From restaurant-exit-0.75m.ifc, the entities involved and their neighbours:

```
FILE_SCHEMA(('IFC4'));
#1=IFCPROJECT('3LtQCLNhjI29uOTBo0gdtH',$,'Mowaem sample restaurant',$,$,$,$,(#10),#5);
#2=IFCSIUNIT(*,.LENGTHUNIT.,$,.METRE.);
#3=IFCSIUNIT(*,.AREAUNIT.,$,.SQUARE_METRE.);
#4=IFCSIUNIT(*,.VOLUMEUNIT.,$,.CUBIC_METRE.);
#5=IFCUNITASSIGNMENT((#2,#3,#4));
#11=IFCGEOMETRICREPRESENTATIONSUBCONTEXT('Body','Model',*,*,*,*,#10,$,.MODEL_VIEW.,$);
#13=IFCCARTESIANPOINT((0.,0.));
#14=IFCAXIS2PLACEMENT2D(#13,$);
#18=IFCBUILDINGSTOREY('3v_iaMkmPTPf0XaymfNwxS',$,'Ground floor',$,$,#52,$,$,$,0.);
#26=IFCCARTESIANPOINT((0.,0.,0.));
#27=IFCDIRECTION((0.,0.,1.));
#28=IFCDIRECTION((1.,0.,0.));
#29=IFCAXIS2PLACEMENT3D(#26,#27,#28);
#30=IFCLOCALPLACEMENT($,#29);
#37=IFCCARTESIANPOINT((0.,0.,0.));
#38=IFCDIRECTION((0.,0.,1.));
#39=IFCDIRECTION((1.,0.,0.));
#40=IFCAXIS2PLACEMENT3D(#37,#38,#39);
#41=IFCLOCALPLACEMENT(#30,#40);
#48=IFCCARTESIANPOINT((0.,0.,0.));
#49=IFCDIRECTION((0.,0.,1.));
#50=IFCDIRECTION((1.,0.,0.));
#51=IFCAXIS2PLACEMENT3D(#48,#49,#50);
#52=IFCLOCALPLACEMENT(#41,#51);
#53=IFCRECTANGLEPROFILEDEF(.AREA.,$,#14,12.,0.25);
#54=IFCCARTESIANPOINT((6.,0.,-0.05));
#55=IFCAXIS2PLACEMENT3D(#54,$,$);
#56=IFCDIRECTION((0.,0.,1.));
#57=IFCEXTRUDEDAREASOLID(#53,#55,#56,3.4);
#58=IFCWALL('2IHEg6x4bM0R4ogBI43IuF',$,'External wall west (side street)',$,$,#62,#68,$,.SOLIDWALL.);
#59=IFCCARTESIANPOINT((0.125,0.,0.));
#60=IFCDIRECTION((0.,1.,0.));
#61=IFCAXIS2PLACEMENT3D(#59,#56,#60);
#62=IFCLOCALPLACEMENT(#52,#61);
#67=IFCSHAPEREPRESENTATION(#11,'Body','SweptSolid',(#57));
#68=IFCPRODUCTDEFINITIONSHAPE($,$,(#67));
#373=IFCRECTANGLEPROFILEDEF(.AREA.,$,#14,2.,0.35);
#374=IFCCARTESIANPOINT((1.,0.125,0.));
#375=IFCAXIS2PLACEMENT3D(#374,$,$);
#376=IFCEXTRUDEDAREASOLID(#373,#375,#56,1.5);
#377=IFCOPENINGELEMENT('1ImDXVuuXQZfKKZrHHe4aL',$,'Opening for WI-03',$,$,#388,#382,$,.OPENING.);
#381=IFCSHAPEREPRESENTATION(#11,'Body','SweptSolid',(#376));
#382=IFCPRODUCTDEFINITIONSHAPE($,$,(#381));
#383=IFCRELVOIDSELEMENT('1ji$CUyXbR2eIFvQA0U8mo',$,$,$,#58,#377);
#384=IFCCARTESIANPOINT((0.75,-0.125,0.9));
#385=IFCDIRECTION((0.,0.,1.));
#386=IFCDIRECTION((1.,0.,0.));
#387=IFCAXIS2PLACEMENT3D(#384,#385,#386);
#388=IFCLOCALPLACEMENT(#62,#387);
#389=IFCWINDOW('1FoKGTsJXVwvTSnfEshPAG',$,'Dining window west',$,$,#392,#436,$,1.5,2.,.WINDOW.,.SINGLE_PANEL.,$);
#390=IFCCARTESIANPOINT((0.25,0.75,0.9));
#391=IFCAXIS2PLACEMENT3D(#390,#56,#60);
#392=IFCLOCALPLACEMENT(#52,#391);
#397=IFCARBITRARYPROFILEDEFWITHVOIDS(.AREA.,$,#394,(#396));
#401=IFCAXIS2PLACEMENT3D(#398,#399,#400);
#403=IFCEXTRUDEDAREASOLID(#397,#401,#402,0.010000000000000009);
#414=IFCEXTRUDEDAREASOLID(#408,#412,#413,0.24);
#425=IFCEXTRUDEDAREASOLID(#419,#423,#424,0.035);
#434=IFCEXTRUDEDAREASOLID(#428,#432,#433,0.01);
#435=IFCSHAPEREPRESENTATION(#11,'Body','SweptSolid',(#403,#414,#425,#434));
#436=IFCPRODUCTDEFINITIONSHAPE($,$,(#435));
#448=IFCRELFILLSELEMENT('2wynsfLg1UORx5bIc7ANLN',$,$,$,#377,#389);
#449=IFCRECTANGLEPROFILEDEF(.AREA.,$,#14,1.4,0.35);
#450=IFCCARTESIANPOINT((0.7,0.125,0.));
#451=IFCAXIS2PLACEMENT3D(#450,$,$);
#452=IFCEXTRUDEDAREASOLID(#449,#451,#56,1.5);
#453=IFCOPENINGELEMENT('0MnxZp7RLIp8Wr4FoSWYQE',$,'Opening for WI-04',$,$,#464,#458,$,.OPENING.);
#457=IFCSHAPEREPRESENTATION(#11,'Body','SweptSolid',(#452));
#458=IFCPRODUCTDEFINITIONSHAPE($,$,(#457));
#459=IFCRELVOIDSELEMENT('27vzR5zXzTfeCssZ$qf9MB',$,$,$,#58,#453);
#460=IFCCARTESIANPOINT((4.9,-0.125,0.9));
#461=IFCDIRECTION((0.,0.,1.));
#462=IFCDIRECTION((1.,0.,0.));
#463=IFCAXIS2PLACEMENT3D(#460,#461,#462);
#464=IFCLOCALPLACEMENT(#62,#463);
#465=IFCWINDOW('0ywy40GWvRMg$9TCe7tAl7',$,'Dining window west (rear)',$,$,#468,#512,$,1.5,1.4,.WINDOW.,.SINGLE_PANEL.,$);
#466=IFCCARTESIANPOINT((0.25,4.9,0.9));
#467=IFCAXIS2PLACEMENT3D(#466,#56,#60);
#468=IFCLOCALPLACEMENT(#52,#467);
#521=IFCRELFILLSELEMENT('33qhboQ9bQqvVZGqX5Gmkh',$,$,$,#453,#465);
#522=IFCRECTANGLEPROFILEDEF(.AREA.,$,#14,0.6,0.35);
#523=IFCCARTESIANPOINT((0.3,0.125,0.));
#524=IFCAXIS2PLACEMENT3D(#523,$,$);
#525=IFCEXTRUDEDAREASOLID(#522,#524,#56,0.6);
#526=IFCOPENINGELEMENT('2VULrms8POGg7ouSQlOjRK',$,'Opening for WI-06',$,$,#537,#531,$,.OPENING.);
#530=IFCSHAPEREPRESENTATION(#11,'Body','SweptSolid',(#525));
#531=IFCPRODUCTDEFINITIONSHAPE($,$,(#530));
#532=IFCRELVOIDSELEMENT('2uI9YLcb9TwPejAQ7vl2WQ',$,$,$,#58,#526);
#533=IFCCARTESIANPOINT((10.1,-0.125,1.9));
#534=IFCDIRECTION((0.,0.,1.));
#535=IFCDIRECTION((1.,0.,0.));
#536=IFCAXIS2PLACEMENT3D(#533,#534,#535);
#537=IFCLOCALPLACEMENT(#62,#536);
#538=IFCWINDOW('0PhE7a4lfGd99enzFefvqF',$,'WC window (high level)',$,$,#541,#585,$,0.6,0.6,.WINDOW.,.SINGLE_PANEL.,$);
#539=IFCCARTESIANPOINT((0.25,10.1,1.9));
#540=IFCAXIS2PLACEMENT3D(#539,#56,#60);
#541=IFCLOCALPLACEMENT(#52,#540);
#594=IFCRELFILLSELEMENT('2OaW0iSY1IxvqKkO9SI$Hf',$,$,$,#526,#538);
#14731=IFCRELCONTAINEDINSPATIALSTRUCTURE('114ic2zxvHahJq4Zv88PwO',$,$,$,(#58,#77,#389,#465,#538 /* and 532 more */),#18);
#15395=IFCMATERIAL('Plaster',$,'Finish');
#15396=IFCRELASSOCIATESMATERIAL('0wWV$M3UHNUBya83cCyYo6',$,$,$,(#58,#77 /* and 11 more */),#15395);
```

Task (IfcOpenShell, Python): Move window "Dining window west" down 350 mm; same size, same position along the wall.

```python
import numpy as np
import ifcopenshell
import ifcopenshell.api.geometry
import ifcopenshell.util.placement
import ifcopenshell.util.unit

model = ifcopenshell.open("restaurant-exit-0.75m.ifc")
unit_scale = ifcopenshell.util.unit.calculate_unit_scale(model)

window = model.by_guid("1FoKGTsJXVwvTSnfEshPAG")
opening = window.FillsVoids[0].RelatingOpeningElement
dz = -0.35 / unit_scale

shift = np.array([0.0, 0.0, dz])
# The window is not placed relative to its opening, so move both.
for product in (opening, window):
    matrix = ifcopenshell.util.placement.get_local_placement(product.ObjectPlacement)
    matrix[:3, 3] += shift
    ifcopenshell.api.geometry.edit_object_placement(model, product=product, matrix=matrix, is_si=False)

print(f"moved by {dz * unit_scale:+.3f} m")

model.write("restaurant-exit-0.75m-out.ifc")
```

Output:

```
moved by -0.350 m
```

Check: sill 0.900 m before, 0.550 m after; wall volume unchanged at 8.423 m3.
